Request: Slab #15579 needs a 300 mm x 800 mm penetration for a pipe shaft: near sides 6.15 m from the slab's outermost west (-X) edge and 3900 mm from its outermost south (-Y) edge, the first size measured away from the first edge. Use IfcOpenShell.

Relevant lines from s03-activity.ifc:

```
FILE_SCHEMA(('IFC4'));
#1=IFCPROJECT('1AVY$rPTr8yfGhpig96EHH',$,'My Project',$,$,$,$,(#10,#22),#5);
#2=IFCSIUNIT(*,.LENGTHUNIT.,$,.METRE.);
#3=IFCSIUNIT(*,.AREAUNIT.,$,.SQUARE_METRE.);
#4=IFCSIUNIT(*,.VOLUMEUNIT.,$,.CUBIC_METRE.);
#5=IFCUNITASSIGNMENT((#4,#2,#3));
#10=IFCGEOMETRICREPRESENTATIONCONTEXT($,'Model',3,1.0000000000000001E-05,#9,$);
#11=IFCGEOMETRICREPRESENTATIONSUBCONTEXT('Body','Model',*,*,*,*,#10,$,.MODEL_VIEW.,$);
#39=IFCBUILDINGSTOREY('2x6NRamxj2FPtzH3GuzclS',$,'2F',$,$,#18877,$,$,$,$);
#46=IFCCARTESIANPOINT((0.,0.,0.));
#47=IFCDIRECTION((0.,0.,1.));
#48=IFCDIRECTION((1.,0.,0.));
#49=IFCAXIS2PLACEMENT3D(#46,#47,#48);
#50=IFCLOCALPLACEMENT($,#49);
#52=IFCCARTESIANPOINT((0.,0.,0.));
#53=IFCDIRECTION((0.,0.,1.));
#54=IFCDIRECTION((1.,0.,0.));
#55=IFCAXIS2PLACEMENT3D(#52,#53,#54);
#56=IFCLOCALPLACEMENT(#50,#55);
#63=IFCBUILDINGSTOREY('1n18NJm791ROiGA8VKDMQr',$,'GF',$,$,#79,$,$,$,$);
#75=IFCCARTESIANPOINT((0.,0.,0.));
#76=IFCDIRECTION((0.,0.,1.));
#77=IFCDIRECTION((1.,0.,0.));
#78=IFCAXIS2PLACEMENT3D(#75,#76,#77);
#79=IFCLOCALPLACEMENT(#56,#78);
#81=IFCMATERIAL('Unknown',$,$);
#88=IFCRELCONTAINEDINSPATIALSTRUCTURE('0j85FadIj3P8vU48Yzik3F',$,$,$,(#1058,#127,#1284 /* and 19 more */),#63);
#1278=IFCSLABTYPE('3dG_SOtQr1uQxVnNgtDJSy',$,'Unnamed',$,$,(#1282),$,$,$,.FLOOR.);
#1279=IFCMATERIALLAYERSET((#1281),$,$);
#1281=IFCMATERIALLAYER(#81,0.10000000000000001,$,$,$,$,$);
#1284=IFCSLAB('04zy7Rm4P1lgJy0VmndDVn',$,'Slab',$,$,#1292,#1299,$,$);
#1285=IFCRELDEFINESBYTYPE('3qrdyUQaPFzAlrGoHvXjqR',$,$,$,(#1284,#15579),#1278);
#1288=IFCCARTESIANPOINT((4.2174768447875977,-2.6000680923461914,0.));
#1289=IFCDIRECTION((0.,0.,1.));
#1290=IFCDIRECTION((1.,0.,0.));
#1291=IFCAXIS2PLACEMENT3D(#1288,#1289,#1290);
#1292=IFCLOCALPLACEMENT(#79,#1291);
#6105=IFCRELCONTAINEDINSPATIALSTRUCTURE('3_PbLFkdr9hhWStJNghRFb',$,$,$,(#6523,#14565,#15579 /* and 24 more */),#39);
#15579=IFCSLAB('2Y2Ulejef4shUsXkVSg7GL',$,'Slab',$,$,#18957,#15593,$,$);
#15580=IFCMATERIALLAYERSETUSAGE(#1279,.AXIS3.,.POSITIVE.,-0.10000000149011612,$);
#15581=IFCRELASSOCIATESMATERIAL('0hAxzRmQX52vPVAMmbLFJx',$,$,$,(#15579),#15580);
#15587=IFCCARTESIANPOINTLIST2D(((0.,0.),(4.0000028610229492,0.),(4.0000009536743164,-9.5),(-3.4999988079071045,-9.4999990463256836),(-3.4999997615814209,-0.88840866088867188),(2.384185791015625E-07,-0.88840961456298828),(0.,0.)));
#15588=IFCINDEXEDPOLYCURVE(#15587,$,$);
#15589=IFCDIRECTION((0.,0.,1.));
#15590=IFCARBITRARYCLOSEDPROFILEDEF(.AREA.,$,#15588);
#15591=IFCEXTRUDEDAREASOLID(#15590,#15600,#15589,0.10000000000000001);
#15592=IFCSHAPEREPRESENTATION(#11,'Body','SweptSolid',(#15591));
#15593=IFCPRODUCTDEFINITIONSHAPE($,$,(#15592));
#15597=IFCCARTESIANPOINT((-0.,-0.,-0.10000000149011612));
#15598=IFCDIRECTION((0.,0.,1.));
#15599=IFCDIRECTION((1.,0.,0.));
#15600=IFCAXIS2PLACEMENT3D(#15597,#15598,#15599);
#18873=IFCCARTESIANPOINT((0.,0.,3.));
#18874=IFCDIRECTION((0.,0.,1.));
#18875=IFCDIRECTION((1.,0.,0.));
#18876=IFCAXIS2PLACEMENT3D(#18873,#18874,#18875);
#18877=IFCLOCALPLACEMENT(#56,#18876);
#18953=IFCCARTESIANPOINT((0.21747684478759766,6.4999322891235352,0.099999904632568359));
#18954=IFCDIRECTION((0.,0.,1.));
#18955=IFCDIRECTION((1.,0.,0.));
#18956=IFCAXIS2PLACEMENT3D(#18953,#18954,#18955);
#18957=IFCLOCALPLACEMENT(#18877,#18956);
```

```python
import numpy as np
import ifcopenshell
import ifcopenshell.api.feature
import ifcopenshell.api.geometry
import ifcopenshell.api.root
import ifcopenshell.geom
import ifcopenshell.util.placement
import ifcopenshell.util.representation
import ifcopenshell.util.shape
import ifcopenshell.util.unit

model = ifcopenshell.open("s03-activity.ifc")
unit_scale = ifcopenshell.util.unit.calculate_unit_scale(model)
settings = ifcopenshell.geom.settings()


def volume(element):
    """Net volume in cubic metres, openings subtracted."""
    shape = ifcopenshell.geom.create_shape(settings, element)
    return ifcopenshell.util.shape.get_volume(shape.geometry)


slab = model.by_guid("2Y2Ulejef4shUsXkVSg7GL")
before = volume(slab)

# Extent in the slab's own axes, in metres. The edges named are its -X and -Y sides.
slab_shape = ifcopenshell.geom.create_shape(settings, slab)
vertices = ifcopenshell.util.shape.get_vertices(slab_shape.geometry)
x_min, y_min, bottom = vertices.min(axis=0)
top = vertices[:, 2].max()

opening = ifcopenshell.api.root.create_entity(model, ifc_class="IfcOpeningElement", name="Pipe shaft opening", predefined_type="OPENING")
context = ifcopenshell.util.representation.get_context(model, "Model", "Body", "MODEL_VIEW")
width, depth = 0.3, 0.8
outline = [(0.0, 0.0), (width, 0.0), (width, depth), (0.0, depth), (0.0, 0.0)]
# Overshoot both faces by 50 mm so the cut is clean.
shape = ifcopenshell.api.geometry.add_slab_representation(
    model, context=context, depth=top - bottom + 0.1, polyline=outline
)
ifcopenshell.api.geometry.assign_representation(model, product=opening, representation=shape)

matrix = ifcopenshell.util.placement.get_local_placement(slab.ObjectPlacement)
matrix[:, 3] = matrix @ np.append(np.array([x_min + 6.15, y_min + 3.9, bottom - 0.05]) / unit_scale, 1.0)
ifcopenshell.api.geometry.edit_object_placement(model, product=opening, matrix=matrix, is_si=False)
ifcopenshell.api.feature.add_feature(model, feature=opening, element=slab)

after = volume(slab)

print(f"slab volume {before:.3f} -> {after:.3f} m3")

model.write("s03-activity_edited.ifc")
```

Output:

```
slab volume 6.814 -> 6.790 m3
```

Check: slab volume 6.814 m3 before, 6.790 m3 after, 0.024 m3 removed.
